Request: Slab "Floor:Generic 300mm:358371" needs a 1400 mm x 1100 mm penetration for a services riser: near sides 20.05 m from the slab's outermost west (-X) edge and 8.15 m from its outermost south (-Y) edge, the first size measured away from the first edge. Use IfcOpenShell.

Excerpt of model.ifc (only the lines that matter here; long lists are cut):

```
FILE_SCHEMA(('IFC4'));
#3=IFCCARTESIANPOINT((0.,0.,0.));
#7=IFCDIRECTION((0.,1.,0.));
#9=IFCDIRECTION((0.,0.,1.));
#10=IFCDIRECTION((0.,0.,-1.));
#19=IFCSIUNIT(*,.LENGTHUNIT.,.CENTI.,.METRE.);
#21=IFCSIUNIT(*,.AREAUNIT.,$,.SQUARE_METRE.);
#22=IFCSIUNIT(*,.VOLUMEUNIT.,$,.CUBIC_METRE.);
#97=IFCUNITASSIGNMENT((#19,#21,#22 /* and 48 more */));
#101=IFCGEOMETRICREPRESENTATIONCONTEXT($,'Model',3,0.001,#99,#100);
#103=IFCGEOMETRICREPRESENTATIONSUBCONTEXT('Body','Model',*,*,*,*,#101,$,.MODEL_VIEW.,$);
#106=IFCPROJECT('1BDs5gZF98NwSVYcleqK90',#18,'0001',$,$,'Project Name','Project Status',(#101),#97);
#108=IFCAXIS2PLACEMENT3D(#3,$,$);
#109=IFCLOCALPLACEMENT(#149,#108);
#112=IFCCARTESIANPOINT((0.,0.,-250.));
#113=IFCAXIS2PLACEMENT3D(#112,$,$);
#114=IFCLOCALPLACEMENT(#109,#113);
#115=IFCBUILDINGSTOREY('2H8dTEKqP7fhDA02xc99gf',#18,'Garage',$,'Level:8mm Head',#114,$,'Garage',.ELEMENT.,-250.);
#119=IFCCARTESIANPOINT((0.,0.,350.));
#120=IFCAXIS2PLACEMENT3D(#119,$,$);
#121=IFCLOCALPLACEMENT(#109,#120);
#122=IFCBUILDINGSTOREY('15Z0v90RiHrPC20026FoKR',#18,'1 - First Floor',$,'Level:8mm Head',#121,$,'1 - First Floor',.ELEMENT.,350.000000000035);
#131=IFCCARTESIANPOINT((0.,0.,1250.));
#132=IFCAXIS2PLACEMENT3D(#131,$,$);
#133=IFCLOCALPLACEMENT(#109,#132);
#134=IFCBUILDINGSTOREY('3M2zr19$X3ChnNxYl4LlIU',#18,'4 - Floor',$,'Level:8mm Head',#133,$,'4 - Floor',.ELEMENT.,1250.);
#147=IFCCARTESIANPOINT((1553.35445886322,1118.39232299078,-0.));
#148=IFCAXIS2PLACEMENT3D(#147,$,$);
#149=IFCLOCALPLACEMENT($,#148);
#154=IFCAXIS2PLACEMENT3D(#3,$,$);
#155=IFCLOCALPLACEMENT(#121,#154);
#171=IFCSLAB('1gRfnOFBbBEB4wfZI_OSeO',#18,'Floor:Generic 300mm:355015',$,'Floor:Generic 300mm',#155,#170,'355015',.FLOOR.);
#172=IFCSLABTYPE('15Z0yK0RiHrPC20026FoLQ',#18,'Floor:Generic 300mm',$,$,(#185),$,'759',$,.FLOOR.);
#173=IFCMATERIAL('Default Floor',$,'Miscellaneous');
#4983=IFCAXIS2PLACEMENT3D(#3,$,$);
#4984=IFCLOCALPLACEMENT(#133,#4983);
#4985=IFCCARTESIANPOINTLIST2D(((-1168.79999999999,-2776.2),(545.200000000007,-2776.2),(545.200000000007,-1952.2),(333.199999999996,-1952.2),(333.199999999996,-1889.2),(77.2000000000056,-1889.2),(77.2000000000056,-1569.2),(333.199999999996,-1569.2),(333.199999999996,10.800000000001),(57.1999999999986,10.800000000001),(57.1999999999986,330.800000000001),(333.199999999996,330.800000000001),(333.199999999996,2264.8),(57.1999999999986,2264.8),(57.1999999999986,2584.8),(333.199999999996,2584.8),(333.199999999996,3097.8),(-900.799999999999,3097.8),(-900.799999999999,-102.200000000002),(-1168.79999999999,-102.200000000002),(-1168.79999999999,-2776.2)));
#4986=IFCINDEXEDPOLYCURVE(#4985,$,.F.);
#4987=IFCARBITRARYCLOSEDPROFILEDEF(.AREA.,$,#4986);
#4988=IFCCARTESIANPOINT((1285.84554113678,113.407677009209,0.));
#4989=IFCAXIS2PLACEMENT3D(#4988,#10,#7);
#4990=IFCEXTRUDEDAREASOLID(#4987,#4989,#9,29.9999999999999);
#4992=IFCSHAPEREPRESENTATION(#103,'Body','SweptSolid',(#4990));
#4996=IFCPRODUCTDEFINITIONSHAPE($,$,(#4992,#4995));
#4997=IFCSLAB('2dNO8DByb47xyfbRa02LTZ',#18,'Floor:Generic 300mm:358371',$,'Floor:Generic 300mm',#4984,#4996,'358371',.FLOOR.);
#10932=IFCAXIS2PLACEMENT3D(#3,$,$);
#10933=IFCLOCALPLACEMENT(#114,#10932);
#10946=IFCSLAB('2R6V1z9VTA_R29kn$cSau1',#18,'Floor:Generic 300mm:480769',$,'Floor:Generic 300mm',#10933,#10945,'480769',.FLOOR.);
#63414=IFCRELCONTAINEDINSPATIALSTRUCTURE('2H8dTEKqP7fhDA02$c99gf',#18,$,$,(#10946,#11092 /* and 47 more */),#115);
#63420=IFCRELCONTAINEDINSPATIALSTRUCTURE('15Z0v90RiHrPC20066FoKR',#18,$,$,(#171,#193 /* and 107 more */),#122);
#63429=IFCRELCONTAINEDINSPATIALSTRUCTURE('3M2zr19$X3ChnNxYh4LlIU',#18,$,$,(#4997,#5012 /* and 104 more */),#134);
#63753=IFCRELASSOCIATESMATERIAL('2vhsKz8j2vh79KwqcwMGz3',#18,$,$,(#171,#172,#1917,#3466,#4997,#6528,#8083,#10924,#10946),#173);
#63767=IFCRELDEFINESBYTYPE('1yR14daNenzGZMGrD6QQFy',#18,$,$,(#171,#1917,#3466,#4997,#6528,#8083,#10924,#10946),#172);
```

```python
import numpy as np
import ifcopenshell
import ifcopenshell.api.feature
import ifcopenshell.api.geometry
import ifcopenshell.api.root
import ifcopenshell.geom
import ifcopenshell.util.placement
import ifcopenshell.util.representation
import ifcopenshell.util.shape
import ifcopenshell.util.unit

model = ifcopenshell.open("model.ifc")
unit_scale = ifcopenshell.util.unit.calculate_unit_scale(model)
settings = ifcopenshell.geom.settings()


def volume(element):
    """Net volume in cubic metres, openings subtracted."""
    shape = ifcopenshell.geom.create_shape(settings, element)
    return ifcopenshell.util.shape.get_volume(shape.geometry)


slab = model.by_guid("2dNO8DByb47xyfbRa02LTZ")
before = volume(slab)

# Extent in the slab's own axes, in metres. The edges named are its -X and -Y sides.
slab_shape = ifcopenshell.geom.create_shape(settings, slab)
vertices = ifcopenshell.util.shape.get_vertices(slab_shape.geometry)
x_min, y_min, bottom = vertices.min(axis=0)
top = vertices[:, 2].max()

opening = ifcopenshell.api.root.create_entity(model, ifc_class="IfcOpeningElement", name="Services riser opening", predefined_type="OPENING")
context = ifcopenshell.util.representation.get_context(model, "Model", "Body", "MODEL_VIEW")
width, depth = 1.4, 1.1
outline = [(0.0, 0.0), (width, 0.0), (width, depth), (0.0, depth), (0.0, 0.0)]
# Overshoot both faces by 50 mm so the cut is clean.
shape = ifcopenshell.api.geometry.add_slab_representation(
    model, context=context, depth=top - bottom + 0.1, polyline=outline
)
ifcopenshell.api.geometry.assign_representation(model, product=opening, representation=shape)

matrix = ifcopenshell.util.placement.get_local_placement(slab.ObjectPlacement)
matrix[:, 3] = matrix @ np.append(np.array([x_min + 20.05, y_min + 8.15, bottom - 0.05]) / unit_scale, 1.0)
ifcopenshell.api.geometry.edit_object_placement(model, product=opening, matrix=matrix, is_si=False)
ifcopenshell.api.feature.add_feature(model, feature=opening, element=slab)

after = volume(slab)

print(f"slab volume {before:.3f} -> {after:.3f} m3")

model.write("model_edited.ifc")
```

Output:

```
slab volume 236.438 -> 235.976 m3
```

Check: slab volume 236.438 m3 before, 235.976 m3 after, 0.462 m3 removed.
